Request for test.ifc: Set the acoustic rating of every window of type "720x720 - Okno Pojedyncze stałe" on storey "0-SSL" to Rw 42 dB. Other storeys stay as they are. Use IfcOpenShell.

First a look at what the model holds.

```python
import ifcopenshell
import ifcopenshell.util.element

model = ifcopenshell.open("test.ifc")
print(model.schema)
storey = next(s for s in model.by_type("IfcBuildingStorey") if s.Name == "0-SSL")
windows = [e for e in ifcopenshell.util.element.get_decomposition(storey) if e.is_a("IfcWindow")]
seen = {}
for e in windows:
    element_type = ifcopenshell.util.element.get_type(e)
    key = (element_type.Name if element_type != e and element_type else None, ifcopenshell.util.element.get_pset(e, "Pset_WindowCommon", "AcousticRating"))
    seen[key] = seen.get(key, 0) + 1
for (name, value), count in sorted(seen.items(), key=str):
    print(count, "x", name, "|", value)
```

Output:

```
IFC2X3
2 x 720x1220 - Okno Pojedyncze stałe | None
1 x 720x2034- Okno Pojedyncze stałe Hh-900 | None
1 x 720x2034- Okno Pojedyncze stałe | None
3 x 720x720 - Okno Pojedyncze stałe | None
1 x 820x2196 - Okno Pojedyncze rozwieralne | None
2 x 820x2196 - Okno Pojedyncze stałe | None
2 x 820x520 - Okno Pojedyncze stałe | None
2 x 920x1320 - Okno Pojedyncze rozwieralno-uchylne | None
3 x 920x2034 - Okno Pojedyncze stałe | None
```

```python
import ifcopenshell
import ifcopenshell.api.pset
import ifcopenshell.util.element

model = ifcopenshell.open("test.ifc")

storey = next(s for s in model.by_type("IfcBuildingStorey") if s.Name == "0-SSL")
windows = [e for e in ifcopenshell.util.element.get_decomposition(storey) if e.is_a("IfcWindow")]

count = 0
for e in windows:
    element_type = ifcopenshell.util.element.get_type(e)
    if element_type in (None, e) or element_type.Name != "720x720 - Okno Pojedyncze stałe":
        continue
    # add_pset returns the element's existing set when there is one.
    pset = ifcopenshell.api.pset.add_pset(model, product=e, name="Pset_WindowCommon")
    ifcopenshell.api.pset.edit_pset(model, pset=pset, properties={"AcousticRating": "Rw 42 dB"})
    count += 1

print(count, "windows updated")

model.write("test_rev.ifc")
```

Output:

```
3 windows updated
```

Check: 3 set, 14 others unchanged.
